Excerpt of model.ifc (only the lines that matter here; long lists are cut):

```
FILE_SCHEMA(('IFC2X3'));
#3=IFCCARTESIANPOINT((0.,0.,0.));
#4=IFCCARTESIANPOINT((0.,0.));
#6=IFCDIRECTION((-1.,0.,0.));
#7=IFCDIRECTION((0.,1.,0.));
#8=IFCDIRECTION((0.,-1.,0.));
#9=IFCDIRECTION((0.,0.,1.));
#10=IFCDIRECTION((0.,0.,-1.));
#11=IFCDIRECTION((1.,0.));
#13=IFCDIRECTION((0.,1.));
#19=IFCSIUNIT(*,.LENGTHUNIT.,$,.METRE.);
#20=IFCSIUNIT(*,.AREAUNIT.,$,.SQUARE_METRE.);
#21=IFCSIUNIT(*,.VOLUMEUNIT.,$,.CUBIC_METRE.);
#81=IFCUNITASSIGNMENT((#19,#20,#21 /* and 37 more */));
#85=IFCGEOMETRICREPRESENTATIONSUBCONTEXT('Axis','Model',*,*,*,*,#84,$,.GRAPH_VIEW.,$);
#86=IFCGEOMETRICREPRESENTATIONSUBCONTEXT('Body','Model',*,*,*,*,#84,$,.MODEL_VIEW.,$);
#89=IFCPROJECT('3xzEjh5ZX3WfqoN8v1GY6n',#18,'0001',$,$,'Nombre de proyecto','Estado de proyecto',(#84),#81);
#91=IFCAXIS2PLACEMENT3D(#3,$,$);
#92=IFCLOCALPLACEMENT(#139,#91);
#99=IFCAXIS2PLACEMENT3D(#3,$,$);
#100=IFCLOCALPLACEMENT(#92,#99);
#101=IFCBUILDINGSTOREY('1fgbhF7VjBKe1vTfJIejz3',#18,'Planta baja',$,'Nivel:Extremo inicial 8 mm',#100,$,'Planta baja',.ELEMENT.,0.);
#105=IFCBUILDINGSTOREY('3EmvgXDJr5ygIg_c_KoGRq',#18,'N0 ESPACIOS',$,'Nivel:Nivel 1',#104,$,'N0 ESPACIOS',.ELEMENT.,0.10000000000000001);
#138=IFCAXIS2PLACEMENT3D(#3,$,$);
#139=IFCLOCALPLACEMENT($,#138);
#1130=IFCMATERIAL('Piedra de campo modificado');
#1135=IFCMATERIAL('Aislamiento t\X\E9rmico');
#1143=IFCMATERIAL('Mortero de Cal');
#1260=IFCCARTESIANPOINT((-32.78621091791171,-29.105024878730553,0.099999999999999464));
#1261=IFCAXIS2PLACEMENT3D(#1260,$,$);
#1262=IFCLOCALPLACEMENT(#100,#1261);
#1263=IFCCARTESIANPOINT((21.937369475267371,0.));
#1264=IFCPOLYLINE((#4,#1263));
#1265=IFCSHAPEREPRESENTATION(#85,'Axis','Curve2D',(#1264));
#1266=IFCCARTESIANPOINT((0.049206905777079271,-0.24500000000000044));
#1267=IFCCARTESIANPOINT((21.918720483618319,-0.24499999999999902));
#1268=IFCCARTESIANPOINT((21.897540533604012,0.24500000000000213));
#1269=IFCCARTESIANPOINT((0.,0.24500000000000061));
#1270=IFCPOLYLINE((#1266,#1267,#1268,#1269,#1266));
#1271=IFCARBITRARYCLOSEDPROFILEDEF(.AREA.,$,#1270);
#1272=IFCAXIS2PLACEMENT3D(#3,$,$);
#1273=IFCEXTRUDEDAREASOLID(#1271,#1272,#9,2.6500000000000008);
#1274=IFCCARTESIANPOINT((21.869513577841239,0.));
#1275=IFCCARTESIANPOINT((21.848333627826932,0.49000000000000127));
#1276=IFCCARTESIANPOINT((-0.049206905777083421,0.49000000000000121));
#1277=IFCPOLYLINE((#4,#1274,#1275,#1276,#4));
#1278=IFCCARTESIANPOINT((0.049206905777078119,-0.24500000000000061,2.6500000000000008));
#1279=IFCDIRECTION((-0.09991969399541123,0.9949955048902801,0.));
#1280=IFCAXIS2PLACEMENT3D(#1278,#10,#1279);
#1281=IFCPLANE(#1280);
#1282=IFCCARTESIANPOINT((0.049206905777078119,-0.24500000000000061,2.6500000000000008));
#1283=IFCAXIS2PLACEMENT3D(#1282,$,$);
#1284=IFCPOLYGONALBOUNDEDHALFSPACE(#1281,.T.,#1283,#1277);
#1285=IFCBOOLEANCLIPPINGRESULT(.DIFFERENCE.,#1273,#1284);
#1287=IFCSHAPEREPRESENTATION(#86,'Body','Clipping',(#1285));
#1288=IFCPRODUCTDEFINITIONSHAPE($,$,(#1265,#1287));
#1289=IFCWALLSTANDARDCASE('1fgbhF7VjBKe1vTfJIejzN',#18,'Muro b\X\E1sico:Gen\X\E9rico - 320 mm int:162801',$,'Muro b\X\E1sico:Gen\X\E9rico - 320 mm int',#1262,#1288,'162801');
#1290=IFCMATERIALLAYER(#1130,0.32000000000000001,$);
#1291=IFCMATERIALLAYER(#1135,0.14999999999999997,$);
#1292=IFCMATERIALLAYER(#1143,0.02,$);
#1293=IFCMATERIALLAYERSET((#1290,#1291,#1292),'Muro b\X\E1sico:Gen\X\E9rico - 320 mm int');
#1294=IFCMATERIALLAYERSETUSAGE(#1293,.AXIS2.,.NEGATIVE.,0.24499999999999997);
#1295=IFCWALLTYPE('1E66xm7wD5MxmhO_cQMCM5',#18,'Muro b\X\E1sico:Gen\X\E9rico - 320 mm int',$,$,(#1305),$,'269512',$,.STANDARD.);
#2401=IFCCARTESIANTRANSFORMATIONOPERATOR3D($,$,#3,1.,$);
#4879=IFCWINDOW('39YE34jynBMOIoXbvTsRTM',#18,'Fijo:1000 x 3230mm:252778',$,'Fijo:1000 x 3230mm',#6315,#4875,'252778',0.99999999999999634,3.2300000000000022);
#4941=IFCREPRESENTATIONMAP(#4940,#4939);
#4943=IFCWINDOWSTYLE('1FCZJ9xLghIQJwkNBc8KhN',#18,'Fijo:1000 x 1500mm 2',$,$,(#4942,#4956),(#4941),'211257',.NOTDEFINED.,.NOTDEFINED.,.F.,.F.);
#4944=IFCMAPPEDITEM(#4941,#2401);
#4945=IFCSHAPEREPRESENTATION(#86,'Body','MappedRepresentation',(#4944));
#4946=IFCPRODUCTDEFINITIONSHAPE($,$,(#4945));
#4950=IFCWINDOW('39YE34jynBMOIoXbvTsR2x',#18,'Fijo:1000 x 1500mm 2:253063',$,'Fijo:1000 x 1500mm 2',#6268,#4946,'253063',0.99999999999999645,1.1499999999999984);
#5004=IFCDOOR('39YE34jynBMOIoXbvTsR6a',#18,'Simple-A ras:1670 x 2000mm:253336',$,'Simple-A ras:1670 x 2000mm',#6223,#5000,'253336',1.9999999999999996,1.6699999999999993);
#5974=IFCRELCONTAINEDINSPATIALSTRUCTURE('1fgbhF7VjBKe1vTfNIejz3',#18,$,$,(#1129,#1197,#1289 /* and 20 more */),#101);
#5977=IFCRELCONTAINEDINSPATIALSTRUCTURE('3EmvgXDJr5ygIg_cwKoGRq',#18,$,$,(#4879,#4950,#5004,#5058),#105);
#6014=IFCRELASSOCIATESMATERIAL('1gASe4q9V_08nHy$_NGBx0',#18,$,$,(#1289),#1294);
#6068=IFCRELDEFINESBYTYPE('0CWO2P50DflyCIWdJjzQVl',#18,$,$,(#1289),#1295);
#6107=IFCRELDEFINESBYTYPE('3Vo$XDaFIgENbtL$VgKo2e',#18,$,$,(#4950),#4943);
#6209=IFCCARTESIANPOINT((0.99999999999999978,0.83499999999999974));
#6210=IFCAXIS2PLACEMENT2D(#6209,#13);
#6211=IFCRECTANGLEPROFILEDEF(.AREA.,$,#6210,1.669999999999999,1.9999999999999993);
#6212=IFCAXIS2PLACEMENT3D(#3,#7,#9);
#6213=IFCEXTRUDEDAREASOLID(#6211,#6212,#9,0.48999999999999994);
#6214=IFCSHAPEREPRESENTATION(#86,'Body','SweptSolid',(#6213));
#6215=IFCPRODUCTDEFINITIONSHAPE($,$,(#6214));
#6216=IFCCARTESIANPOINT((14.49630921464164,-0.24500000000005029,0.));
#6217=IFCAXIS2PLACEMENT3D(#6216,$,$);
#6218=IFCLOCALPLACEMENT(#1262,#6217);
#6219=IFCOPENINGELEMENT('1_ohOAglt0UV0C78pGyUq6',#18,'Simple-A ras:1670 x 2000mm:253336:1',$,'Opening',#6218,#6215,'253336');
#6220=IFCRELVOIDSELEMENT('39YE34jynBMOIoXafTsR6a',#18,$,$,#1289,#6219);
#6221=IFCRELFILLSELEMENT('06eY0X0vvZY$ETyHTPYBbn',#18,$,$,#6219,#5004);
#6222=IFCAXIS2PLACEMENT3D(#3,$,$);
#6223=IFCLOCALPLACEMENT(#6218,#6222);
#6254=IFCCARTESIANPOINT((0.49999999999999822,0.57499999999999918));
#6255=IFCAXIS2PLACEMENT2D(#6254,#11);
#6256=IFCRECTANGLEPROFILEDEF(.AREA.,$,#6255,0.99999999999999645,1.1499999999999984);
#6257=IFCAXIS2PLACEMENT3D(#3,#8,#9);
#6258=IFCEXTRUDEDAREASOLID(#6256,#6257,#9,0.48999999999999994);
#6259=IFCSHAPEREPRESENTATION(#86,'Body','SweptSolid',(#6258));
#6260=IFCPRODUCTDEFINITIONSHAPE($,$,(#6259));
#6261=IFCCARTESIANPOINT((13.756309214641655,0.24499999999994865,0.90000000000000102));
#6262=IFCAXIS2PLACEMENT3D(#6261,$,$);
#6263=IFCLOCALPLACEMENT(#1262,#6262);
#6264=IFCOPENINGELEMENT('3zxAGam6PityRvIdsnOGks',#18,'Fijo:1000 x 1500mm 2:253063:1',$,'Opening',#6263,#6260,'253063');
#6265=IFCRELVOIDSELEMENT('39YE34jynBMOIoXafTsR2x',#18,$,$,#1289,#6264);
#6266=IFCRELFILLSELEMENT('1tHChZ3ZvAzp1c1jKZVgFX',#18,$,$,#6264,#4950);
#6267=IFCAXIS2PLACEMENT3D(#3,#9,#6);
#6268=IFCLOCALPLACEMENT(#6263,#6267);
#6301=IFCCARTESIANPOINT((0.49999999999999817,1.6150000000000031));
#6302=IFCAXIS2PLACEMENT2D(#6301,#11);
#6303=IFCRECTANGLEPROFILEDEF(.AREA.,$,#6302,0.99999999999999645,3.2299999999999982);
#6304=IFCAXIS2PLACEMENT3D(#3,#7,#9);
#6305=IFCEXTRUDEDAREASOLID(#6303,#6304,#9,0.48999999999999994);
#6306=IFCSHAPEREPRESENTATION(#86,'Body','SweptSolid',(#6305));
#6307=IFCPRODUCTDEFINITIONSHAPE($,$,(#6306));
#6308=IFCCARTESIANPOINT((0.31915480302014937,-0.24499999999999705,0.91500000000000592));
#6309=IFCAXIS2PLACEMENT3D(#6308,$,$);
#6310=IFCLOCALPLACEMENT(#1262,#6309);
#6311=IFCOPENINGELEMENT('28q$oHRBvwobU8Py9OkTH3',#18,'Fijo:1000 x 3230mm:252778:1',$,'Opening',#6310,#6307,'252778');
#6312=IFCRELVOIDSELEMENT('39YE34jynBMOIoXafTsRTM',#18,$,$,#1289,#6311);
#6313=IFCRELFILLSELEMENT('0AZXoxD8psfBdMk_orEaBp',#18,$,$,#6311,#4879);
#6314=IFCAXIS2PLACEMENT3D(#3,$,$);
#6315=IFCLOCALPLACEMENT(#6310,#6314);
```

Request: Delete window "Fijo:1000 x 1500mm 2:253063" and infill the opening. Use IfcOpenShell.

```python
import ifcopenshell
import ifcopenshell.api.feature
import ifcopenshell.api.root
import ifcopenshell.geom
import ifcopenshell.util.shape

model = ifcopenshell.open("model.ifc")
settings = ifcopenshell.geom.settings()


def volume(element):
    """Net volume in cubic metres, openings subtracted."""
    shape = ifcopenshell.geom.create_shape(settings, element)
    return ifcopenshell.util.shape.get_volume(shape.geometry)


window = model.by_id(4950)
opening = window.FillsVoids[0].RelatingOpeningElement
wall = opening.VoidsElements[0].RelatingBuildingElement
before = volume(wall)

ifcopenshell.api.root.remove_product(model, product=window)
ifcopenshell.api.feature.remove_feature(model, feature=opening)

after = volume(wall)

print(f"wall volume {before:.3f} -> {after:.3f} m3")

model.write("model_v2.ifc")
```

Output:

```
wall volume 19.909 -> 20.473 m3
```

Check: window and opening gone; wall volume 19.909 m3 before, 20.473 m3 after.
